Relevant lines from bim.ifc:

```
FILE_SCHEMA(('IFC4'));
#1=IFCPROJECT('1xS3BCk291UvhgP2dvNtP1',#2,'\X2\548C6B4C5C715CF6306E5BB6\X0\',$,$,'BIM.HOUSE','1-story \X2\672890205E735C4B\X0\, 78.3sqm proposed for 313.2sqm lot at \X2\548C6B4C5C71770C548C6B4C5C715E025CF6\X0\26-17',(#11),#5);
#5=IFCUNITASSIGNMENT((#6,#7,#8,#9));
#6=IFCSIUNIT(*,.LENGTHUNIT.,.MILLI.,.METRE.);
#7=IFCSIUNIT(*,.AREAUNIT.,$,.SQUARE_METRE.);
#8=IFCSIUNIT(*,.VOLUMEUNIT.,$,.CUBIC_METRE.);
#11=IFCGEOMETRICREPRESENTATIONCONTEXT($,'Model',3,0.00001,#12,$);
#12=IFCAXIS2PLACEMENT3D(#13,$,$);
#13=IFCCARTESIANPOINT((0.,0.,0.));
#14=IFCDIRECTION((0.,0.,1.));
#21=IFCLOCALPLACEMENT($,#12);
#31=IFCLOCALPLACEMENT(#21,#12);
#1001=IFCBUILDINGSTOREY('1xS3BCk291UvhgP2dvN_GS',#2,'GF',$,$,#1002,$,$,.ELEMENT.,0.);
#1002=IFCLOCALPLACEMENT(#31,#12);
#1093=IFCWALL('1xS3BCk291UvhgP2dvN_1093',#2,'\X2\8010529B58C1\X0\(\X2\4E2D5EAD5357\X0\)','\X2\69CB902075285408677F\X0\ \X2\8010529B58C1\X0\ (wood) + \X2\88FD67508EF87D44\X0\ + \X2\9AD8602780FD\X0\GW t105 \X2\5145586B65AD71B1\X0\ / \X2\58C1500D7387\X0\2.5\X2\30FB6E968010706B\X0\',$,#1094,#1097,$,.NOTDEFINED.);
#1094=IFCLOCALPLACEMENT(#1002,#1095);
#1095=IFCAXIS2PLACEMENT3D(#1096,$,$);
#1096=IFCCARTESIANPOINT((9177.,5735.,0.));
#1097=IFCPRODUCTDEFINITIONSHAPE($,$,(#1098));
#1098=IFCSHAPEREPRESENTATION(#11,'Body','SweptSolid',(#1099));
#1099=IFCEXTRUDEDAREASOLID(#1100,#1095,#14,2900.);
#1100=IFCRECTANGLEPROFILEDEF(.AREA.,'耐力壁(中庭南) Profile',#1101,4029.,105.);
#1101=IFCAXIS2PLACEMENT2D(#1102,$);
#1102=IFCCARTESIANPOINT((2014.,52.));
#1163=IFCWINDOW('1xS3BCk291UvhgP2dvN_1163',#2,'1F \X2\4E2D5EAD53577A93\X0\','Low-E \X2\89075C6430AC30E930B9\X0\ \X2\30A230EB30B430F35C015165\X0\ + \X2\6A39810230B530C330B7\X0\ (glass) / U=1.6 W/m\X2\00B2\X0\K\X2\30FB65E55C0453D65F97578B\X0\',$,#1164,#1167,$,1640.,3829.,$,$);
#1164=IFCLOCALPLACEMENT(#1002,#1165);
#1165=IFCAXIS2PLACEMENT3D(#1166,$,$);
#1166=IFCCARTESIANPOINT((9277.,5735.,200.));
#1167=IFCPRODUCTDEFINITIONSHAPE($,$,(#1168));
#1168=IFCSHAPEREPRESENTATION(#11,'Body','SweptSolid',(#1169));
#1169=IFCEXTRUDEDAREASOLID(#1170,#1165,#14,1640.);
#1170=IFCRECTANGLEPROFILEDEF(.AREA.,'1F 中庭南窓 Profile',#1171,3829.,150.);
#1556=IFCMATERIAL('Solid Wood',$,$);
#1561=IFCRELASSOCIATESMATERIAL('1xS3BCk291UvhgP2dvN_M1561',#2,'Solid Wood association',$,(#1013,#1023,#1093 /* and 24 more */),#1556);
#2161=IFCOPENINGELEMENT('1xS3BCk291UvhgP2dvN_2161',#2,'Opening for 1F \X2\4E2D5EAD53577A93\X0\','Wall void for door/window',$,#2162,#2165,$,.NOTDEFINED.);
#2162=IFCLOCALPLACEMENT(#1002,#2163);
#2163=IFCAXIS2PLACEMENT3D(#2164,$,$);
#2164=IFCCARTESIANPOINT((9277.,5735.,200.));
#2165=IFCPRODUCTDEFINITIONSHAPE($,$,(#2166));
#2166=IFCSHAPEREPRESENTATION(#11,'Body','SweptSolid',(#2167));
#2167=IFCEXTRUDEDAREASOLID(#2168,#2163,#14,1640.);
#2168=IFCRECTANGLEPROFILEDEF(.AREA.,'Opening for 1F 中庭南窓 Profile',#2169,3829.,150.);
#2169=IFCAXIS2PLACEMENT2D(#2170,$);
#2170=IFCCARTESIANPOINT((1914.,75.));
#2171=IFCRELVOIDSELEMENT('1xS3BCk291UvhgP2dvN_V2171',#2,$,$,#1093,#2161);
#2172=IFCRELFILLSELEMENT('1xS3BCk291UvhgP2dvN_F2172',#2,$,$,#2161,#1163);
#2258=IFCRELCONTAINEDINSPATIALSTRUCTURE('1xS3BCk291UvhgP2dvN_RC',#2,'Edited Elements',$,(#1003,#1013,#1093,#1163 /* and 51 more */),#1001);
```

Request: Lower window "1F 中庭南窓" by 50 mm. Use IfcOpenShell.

```python
import numpy as np
import ifcopenshell
import ifcopenshell.api.geometry
import ifcopenshell.util.placement
import ifcopenshell.util.unit

model = ifcopenshell.open("bim.ifc")
unit_scale = ifcopenshell.util.unit.calculate_unit_scale(model)

window = model.by_id(1163)
opening = window.FillsVoids[0].RelatingOpeningElement
dz = -0.05 / unit_scale

shift = np.array([0.0, 0.0, dz])
# The window is not placed relative to its opening, so move both.
for product in (opening, window):
    matrix = ifcopenshell.util.placement.get_local_placement(product.ObjectPlacement)
    matrix[:3, 3] += shift
    ifcopenshell.api.geometry.edit_object_placement(model, product=product, matrix=matrix, is_si=False)

print(f"moved by {dz * unit_scale:+.3f} m")

model.write("bim_edited.ifc")
```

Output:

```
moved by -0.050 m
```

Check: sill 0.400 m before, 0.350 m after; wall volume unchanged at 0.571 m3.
